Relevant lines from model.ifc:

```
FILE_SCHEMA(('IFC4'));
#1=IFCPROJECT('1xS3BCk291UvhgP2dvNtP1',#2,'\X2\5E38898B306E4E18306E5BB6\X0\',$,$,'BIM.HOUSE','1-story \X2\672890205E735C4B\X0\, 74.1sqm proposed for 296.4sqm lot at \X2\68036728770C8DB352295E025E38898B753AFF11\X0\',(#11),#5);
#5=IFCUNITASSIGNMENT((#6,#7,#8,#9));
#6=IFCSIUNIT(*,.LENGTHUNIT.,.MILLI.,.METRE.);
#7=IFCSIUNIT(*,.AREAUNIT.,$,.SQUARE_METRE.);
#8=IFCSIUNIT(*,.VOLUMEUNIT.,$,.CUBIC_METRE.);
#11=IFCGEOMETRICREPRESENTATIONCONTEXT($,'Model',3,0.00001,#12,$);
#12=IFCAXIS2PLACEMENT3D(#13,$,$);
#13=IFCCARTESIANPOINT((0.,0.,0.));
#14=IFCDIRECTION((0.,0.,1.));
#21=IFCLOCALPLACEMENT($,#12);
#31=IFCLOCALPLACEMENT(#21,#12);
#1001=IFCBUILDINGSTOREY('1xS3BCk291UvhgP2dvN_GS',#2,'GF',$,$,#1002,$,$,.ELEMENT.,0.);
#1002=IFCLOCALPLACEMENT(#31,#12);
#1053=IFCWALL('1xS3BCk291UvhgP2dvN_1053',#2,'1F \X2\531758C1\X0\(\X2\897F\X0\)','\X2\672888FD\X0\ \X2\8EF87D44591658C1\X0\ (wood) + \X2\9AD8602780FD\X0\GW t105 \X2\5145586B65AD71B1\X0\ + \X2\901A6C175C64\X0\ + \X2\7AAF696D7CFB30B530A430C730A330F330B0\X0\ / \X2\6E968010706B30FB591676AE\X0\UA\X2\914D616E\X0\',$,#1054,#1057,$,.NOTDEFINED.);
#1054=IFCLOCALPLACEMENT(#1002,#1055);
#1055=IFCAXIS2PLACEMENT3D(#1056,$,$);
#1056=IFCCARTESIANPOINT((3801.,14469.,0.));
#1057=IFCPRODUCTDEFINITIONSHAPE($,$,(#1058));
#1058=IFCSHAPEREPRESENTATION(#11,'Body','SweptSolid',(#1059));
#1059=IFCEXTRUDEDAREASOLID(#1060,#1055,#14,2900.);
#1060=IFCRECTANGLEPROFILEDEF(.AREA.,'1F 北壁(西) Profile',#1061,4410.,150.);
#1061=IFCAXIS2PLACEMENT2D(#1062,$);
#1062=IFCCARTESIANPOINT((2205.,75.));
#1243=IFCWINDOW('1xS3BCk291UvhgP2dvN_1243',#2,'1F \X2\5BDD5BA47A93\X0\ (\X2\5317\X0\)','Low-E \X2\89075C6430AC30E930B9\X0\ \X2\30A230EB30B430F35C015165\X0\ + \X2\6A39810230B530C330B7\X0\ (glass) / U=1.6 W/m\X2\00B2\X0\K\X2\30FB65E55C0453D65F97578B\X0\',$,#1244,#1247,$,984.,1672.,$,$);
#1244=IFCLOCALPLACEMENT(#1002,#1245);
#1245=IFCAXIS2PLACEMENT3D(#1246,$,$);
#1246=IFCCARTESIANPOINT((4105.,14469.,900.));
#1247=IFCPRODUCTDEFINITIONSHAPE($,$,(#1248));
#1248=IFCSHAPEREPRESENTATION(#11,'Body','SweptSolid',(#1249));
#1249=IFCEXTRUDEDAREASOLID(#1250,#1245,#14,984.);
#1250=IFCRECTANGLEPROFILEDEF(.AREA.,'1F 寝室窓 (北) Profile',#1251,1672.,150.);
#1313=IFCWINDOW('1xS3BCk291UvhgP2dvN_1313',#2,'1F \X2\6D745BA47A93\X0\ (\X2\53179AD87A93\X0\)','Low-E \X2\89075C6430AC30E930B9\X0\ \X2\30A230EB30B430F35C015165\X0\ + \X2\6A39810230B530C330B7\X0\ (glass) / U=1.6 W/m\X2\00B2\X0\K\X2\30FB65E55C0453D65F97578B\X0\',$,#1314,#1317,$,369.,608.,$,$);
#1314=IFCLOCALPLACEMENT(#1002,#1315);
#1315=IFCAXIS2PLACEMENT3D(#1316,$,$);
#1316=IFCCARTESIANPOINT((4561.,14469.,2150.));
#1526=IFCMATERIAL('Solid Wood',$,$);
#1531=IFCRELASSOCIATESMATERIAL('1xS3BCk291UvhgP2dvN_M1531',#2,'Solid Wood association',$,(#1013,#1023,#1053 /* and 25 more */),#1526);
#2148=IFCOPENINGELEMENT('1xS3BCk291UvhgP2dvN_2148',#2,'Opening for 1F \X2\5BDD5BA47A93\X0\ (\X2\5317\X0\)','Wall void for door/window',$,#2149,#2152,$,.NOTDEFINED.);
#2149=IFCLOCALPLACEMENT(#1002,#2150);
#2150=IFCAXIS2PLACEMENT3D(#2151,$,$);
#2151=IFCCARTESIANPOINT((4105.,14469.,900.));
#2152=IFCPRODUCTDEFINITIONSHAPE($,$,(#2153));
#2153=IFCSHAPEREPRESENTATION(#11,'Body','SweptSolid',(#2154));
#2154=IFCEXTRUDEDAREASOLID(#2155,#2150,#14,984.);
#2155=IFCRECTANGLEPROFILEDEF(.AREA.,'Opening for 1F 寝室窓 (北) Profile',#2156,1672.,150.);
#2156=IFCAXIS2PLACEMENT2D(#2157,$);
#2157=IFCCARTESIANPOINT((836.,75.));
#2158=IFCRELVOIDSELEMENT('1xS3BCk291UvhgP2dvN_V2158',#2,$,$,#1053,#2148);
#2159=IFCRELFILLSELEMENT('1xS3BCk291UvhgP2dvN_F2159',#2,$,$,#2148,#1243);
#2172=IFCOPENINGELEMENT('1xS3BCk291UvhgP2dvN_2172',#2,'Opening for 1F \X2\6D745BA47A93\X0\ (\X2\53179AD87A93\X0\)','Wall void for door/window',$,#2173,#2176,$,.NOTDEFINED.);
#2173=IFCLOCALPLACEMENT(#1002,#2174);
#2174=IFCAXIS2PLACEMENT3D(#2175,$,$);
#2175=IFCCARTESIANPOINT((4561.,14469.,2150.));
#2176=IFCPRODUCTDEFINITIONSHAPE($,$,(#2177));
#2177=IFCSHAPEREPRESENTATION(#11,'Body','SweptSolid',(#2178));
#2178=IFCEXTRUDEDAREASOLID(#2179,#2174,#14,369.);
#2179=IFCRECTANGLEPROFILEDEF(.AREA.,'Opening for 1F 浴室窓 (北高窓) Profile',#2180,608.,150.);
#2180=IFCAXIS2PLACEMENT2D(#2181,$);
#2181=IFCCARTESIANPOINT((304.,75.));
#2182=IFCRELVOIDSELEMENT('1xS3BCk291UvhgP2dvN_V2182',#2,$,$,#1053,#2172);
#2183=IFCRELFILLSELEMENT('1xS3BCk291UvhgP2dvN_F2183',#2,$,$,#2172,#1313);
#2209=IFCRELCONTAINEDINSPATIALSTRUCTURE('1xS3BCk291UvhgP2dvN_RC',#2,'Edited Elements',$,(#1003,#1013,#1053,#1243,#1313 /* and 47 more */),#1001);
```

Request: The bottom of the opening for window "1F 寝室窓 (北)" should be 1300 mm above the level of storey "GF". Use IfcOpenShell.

```python
import numpy as np
import ifcopenshell
import ifcopenshell.api.geometry
import ifcopenshell.geom
import ifcopenshell.util.element
import ifcopenshell.util.placement
import ifcopenshell.util.shape
import ifcopenshell.util.unit

model = ifcopenshell.open("model.ifc")
unit_scale = ifcopenshell.util.unit.calculate_unit_scale(model)

window = model.by_guid("1xS3BCk291UvhgP2dvN_1243")
opening = window.FillsVoids[0].RelatingOpeningElement
storey = ifcopenshell.util.element.get_container(window, ifc_class="IfcBuildingStorey")
level = ifcopenshell.util.placement.get_local_placement(storey.ObjectPlacement)[2, 3]

# The opening's origin need not be at the sill, so measure its lowest point.
shape = ifcopenshell.geom.create_shape(ifcopenshell.geom.settings(), opening)
bottom = ifcopenshell.util.shape.get_shape_bottom_elevation(shape, shape.geometry) / unit_scale
dz = level + 1.3 / unit_scale - bottom

shift = np.array([0.0, 0.0, dz])
# The window is not placed relative to its opening, so move both.
for product in (opening, window):
    matrix = ifcopenshell.util.placement.get_local_placement(product.ObjectPlacement)
    matrix[:3, 3] += shift
    ifcopenshell.api.geometry.edit_object_placement(model, product=product, matrix=matrix, is_si=False)

print(f"moved by {dz * unit_scale:+.3f} m")

model.write("model_v2.ifc")
```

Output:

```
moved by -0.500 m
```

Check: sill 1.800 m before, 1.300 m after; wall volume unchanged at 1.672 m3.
